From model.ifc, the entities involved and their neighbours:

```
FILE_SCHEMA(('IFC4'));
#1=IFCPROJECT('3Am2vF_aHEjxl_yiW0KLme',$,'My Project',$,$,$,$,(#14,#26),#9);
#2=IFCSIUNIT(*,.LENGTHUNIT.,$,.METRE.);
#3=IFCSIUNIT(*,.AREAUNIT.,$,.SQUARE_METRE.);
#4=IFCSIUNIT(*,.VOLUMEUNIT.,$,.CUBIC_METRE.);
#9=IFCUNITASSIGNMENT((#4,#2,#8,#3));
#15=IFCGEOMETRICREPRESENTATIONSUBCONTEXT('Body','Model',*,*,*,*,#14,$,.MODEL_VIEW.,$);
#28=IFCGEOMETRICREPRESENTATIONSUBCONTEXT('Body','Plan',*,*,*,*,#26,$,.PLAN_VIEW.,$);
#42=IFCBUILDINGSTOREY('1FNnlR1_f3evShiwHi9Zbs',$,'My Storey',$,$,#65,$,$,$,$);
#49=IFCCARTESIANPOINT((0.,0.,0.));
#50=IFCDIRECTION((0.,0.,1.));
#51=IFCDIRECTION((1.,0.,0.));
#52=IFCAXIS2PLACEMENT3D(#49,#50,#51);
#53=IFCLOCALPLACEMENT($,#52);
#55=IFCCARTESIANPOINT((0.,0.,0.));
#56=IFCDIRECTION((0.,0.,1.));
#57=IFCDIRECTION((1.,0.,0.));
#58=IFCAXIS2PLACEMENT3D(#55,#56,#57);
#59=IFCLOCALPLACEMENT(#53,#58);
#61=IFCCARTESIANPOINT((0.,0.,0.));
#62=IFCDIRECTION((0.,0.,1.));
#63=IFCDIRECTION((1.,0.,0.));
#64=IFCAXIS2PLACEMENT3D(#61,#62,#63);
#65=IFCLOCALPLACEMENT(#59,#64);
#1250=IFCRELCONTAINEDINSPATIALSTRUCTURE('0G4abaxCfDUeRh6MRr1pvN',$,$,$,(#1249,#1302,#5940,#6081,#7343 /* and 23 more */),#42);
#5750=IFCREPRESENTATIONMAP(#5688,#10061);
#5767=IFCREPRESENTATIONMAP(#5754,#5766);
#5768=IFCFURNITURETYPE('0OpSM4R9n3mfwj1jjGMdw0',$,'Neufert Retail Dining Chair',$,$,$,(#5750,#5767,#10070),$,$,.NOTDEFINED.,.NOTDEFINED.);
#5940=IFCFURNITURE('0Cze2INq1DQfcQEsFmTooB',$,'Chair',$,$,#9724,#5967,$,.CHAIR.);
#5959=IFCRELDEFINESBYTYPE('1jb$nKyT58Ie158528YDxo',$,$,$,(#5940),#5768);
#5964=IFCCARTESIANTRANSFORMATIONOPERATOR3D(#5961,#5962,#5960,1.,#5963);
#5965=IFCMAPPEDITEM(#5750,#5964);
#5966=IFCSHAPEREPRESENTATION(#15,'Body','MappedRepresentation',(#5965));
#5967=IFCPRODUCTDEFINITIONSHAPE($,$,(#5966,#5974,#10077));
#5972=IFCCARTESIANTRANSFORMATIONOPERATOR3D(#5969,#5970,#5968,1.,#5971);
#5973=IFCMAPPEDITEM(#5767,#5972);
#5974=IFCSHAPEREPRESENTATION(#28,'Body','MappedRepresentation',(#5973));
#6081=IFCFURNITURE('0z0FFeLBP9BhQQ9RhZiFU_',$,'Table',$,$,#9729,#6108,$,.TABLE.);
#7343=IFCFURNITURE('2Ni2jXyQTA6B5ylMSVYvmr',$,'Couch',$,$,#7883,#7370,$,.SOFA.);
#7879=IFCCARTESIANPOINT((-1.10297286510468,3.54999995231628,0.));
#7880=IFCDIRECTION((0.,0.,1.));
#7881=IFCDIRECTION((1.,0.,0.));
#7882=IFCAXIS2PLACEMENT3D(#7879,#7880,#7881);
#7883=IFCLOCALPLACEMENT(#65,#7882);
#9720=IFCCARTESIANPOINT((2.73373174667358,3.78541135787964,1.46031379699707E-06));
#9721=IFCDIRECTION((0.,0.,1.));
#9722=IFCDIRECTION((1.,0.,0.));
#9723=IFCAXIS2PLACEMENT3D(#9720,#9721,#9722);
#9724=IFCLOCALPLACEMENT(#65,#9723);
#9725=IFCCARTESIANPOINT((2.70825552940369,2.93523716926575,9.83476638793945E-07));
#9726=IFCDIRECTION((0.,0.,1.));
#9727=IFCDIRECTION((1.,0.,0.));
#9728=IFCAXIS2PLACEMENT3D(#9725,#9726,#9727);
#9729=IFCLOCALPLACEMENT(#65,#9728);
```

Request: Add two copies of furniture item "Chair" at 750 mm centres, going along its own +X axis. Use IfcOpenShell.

```python
import ifcopenshell
import ifcopenshell.api.geometry
import ifcopenshell.api.root
import ifcopenshell.util.element
import ifcopenshell.util.placement

model = ifcopenshell.open("model.ifc")

source = model.by_id(5940)
base = ifcopenshell.util.placement.get_local_placement(source.ObjectPlacement)
step = base[:3, 0] * 0.75

for i in range(1, 3):
    copy = ifcopenshell.api.root.copy_class(model, product=source)
    copy.Representation = ifcopenshell.util.element.copy_deep(
        model, source.Representation, exclude=["IfcGeometricRepresentationContext", "IfcRepresentationMap"]
    )
    matrix = base.copy()
    matrix[:3, 3] += i * step
    print("added at", matrix[:3, 3].round(3) + 0.0)
    ifcopenshell.api.geometry.edit_object_placement(model, product=copy, matrix=matrix, is_si=False)

model.write("model_edited.ifc")
```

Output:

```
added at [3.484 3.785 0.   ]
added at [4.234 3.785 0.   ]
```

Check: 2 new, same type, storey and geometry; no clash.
